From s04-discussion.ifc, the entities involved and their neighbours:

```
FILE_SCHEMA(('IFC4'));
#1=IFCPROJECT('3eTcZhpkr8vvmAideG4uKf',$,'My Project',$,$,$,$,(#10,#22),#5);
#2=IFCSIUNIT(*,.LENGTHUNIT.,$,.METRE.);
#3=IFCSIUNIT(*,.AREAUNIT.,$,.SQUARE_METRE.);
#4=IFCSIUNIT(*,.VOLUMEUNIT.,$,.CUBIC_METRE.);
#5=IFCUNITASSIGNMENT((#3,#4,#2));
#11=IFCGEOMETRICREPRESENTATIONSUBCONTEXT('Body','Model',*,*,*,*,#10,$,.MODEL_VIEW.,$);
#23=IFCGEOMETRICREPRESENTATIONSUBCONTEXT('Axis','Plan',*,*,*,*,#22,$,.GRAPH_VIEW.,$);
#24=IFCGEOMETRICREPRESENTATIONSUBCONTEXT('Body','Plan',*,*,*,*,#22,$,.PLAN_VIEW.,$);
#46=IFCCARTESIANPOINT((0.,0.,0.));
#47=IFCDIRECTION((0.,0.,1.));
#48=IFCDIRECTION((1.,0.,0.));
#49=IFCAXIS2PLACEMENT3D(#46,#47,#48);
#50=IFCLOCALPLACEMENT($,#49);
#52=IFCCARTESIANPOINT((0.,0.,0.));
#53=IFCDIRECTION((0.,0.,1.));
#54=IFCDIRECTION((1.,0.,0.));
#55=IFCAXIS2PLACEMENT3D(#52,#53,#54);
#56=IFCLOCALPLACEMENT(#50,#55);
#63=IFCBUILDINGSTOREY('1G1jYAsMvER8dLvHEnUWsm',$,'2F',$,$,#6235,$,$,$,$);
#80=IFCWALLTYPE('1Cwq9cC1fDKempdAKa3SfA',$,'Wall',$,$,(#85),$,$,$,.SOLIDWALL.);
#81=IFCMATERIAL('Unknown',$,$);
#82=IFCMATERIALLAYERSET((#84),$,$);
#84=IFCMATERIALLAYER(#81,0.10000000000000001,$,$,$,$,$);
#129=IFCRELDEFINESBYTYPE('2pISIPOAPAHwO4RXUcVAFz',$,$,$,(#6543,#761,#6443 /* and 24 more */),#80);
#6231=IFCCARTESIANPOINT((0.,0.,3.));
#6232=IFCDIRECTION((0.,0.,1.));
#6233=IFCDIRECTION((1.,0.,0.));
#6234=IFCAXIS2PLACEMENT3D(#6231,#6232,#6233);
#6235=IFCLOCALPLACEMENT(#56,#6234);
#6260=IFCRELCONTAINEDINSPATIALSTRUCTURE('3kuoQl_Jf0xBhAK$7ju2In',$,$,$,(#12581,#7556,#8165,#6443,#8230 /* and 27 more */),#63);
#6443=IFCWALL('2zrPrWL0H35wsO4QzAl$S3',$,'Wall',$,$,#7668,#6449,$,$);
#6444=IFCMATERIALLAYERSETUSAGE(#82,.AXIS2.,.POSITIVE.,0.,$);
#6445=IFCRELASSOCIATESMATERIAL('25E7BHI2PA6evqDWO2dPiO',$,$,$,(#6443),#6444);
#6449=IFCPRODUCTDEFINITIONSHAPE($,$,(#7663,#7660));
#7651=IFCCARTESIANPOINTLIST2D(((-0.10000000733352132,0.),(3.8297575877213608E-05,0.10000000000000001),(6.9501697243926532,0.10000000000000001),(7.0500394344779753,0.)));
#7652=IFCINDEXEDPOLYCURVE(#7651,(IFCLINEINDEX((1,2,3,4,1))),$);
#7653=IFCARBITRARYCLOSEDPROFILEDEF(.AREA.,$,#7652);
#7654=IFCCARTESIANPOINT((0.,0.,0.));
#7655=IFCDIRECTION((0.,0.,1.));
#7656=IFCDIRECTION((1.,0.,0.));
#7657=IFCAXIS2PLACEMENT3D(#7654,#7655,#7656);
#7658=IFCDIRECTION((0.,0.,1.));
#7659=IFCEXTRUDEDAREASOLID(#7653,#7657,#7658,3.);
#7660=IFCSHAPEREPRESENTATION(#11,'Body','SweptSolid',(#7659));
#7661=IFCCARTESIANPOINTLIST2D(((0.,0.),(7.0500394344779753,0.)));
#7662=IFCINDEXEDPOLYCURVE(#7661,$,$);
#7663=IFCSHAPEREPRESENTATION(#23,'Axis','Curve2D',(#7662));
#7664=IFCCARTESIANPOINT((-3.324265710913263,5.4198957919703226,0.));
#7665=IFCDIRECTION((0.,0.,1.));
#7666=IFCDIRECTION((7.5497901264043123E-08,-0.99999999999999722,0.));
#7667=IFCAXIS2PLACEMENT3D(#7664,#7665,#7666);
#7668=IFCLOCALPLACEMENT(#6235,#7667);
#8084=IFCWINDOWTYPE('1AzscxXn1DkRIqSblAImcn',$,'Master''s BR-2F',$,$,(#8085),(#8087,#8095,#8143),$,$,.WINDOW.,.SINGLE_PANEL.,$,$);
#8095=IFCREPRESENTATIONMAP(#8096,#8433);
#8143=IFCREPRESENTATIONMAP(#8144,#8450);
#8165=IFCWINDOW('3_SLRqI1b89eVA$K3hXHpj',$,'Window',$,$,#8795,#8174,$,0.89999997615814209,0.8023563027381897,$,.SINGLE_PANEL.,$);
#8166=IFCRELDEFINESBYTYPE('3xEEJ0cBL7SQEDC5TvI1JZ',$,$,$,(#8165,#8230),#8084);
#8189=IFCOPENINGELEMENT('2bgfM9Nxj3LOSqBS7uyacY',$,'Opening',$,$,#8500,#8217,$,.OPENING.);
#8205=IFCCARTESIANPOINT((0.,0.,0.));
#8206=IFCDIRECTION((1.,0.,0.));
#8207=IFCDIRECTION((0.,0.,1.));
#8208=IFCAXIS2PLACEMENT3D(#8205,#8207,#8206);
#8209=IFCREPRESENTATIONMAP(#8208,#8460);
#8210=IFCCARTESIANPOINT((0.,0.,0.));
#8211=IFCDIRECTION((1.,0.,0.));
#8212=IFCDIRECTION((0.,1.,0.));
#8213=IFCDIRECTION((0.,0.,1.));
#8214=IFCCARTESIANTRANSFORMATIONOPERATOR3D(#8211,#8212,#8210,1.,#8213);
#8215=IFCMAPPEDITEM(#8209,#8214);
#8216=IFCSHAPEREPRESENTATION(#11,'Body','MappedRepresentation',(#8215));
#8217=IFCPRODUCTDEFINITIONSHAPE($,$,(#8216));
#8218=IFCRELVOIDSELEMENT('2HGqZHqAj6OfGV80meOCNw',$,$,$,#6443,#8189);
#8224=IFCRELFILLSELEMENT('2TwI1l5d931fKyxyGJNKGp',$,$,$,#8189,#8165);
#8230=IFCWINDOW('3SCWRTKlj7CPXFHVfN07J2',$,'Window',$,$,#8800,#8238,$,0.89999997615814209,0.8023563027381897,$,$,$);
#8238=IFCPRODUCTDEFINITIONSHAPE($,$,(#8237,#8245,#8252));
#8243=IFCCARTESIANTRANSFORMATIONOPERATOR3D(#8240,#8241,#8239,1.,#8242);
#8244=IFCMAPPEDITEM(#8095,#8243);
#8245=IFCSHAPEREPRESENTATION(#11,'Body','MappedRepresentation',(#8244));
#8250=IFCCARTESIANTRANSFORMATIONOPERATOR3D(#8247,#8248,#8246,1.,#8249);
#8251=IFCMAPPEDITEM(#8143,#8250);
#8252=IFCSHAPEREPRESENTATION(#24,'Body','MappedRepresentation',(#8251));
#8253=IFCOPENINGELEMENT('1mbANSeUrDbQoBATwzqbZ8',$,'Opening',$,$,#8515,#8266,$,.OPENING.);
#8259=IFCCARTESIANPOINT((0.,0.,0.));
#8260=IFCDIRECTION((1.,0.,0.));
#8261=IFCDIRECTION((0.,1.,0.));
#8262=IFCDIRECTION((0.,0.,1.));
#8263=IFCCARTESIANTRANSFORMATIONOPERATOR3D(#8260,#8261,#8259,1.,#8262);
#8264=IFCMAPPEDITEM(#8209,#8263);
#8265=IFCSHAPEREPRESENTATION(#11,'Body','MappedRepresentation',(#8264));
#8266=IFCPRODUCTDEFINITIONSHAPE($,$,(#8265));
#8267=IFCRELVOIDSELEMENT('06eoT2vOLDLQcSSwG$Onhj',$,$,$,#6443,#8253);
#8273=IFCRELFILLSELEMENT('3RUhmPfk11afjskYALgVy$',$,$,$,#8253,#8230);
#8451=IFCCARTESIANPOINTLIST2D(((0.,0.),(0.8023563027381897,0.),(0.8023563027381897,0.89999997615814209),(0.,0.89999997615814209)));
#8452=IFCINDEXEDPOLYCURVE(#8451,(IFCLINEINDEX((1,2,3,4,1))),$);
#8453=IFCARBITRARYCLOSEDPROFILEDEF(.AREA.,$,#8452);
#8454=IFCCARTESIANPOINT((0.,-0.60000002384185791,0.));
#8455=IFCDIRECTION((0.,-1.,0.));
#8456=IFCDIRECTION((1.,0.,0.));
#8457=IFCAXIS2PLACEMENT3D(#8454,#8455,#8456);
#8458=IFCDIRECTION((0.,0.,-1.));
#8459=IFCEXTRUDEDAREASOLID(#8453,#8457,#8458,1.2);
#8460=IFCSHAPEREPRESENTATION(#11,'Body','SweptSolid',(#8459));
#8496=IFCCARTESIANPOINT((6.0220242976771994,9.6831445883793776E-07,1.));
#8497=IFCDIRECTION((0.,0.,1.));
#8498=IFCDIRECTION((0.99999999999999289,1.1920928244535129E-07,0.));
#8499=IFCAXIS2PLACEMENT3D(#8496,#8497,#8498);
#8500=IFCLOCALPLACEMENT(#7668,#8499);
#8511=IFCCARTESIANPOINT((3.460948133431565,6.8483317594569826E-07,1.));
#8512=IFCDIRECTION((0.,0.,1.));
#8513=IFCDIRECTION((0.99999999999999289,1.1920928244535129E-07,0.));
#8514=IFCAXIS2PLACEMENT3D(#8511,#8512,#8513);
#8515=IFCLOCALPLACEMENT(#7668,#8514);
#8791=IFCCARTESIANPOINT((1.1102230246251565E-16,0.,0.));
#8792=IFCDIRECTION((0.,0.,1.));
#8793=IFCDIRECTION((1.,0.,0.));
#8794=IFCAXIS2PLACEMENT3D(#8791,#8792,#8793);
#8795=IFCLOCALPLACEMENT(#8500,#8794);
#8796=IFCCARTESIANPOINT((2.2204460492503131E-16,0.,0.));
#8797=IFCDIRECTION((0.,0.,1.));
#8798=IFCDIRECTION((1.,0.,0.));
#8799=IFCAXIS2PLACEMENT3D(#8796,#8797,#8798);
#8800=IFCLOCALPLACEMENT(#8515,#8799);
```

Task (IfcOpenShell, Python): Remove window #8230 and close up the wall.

```python
import ifcopenshell
import ifcopenshell.api.feature
import ifcopenshell.api.root
import ifcopenshell.geom
import ifcopenshell.util.shape

model = ifcopenshell.open("s04-discussion.ifc")
settings = ifcopenshell.geom.settings()


def volume(element):
    """Net volume in cubic metres, openings subtracted."""
    shape = ifcopenshell.geom.create_shape(settings, element)
    return ifcopenshell.util.shape.get_volume(shape.geometry)


window = model.by_guid("3SCWRTKlj7CPXFHVfN07J2")
opening = window.FillsVoids[0].RelatingOpeningElement
wall = opening.VoidsElements[0].RelatingBuildingElement
before = volume(wall)

ifcopenshell.api.root.remove_product(model, product=window)
ifcopenshell.api.feature.remove_feature(model, feature=opening)

after = volume(wall)

print(f"wall volume {before:.3f} -> {after:.3f} m3")

model.write("s04-discussion_v2.ifc")
```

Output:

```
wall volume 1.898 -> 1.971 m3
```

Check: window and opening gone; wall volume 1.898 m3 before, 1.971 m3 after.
